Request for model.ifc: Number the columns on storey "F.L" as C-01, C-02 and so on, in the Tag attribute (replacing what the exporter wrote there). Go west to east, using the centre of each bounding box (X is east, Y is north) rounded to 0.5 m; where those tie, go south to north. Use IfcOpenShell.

First a look at what the model holds.

```python
import ifcopenshell
import ifcopenshell.util.element
import ifcopenshell.util.placement

model = ifcopenshell.open("model.ifc")
print(model.schema)
storey = next(s for s in model.by_type("IfcBuildingStorey") if s.Name == "F.L")
columns = [e for e in ifcopenshell.util.element.get_decomposition(storey) if e.is_a("IfcColumn")]
for e in sorted(columns, key=lambda e: e.id()):
    origin = ifcopenshell.util.placement.get_local_placement(e.ObjectPlacement)[:3, 3]
    print(e.id(), e.Tag, e.Name, origin.round(2) + 0.0, sep=" | ")
```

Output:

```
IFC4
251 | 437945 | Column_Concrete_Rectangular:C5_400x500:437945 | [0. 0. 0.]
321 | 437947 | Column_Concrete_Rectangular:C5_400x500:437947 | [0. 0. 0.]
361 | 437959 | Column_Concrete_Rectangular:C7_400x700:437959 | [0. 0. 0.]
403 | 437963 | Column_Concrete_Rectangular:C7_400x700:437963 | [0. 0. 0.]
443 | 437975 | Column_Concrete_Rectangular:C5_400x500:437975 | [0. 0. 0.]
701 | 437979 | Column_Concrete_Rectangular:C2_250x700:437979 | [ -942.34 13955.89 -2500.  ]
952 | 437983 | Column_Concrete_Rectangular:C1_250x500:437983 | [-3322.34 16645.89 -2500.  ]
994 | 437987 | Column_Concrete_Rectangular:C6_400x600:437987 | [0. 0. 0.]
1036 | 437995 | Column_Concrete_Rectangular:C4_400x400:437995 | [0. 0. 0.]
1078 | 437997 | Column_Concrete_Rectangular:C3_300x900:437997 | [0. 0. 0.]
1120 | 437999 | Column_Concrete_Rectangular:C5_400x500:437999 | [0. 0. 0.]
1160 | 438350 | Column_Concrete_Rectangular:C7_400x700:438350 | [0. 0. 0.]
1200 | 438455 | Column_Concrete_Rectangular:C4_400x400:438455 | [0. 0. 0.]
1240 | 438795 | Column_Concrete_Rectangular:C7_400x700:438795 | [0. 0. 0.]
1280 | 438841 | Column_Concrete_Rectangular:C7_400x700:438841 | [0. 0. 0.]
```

```python
import ifcopenshell
import ifcopenshell.geom
import ifcopenshell.util.element
import ifcopenshell.util.shape

model = ifcopenshell.open("model.ifc")
settings = ifcopenshell.geom.settings()
settings.set("use-world-coords", True)


def centre(element):
    shape = ifcopenshell.geom.create_shape(settings, element)
    return ifcopenshell.util.shape.get_bbox_centroid(shape.geometry)


storey = next(s for s in model.by_type("IfcBuildingStorey") if s.Name == "F.L")
columns = [e for e in ifcopenshell.util.element.get_decomposition(storey) if e.is_a("IfcColumn")]

# Insertion points can sit at a corner or the storey origin, so sort by the geometry (in metres).
centres = {e: centre(e) for e in columns}
columns.sort(key=lambda e: (round(centres[e][0] / 0.5), centres[e][1]))

for i, e in enumerate(columns, start=1):
    number = f"C-{i:02d}"
    e.Tag = number
    print(e.id(), number)

model.write("model_v2.ifc")
```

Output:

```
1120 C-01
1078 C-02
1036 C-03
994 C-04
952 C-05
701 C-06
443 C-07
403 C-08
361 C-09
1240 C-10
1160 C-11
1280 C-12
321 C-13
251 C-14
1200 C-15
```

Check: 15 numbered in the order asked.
